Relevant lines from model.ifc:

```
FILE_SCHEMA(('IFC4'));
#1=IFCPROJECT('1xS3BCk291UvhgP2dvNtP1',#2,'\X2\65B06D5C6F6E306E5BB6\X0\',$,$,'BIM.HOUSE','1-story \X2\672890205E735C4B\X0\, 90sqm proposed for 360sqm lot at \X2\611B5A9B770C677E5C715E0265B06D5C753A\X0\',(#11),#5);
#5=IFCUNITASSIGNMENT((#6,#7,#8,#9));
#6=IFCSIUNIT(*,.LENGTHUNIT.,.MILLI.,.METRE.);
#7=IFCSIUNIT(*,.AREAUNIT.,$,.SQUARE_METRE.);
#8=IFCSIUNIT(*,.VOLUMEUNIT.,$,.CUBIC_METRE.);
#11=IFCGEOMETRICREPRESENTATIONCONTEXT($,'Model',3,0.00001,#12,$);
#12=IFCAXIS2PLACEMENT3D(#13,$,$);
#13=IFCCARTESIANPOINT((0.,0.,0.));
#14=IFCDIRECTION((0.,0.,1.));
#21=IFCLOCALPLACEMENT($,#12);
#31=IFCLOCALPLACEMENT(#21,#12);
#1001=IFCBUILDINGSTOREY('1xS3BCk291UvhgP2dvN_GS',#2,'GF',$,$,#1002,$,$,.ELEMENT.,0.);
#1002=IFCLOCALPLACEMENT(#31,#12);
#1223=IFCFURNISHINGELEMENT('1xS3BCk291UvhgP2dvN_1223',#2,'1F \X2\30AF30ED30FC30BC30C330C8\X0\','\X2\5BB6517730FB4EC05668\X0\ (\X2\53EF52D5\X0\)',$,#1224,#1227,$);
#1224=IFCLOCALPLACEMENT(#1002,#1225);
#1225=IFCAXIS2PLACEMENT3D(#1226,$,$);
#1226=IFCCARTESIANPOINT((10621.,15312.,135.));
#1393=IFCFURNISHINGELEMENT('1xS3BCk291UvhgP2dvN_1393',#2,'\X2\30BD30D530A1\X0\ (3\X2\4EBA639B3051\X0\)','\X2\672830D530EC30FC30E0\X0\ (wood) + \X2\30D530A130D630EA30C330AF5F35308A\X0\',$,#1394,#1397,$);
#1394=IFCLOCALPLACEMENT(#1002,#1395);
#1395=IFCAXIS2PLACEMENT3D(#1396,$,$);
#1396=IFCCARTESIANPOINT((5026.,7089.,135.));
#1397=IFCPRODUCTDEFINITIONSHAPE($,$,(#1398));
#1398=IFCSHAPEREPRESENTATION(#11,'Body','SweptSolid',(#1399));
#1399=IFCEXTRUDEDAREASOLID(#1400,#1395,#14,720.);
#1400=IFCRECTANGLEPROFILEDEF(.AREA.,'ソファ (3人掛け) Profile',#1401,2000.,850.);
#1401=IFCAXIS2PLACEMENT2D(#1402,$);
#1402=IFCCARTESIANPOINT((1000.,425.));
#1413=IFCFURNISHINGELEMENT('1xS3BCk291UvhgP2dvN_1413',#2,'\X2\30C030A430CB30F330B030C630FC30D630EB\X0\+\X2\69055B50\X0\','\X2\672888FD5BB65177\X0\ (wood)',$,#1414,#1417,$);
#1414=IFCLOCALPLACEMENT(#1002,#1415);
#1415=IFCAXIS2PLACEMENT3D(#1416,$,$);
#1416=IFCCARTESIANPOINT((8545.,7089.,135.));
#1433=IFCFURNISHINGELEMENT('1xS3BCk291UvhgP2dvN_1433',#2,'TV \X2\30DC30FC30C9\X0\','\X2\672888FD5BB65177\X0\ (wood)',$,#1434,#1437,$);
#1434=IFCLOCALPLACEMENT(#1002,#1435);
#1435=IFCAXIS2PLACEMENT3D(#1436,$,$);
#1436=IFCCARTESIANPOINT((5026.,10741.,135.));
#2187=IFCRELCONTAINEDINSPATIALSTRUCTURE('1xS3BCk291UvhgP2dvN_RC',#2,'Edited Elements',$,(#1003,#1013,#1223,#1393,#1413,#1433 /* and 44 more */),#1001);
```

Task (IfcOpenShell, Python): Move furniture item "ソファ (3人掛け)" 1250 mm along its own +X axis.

```python
import ifcopenshell
import ifcopenshell.api.geometry
import ifcopenshell.util.placement
import ifcopenshell.util.unit

model = ifcopenshell.open("model.ifc")
unit_scale = ifcopenshell.util.unit.calculate_unit_scale(model)

item = model.by_guid("1xS3BCk291UvhgP2dvN_1393")
matrix = ifcopenshell.util.placement.get_local_placement(item.ObjectPlacement)
matrix[:3, 3] += matrix[:3, 0] * 1.25 / unit_scale
ifcopenshell.api.geometry.edit_object_placement(model, product=item, matrix=matrix, is_si=False)

print(ifcopenshell.util.placement.get_local_placement(item.ObjectPlacement).round(3) + 0.0)

model.write("model_v2.ifc")
```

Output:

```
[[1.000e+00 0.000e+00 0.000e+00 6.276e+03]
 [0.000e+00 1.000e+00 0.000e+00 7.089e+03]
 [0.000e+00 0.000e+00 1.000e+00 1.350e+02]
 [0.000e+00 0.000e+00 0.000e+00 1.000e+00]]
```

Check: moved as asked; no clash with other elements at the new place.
